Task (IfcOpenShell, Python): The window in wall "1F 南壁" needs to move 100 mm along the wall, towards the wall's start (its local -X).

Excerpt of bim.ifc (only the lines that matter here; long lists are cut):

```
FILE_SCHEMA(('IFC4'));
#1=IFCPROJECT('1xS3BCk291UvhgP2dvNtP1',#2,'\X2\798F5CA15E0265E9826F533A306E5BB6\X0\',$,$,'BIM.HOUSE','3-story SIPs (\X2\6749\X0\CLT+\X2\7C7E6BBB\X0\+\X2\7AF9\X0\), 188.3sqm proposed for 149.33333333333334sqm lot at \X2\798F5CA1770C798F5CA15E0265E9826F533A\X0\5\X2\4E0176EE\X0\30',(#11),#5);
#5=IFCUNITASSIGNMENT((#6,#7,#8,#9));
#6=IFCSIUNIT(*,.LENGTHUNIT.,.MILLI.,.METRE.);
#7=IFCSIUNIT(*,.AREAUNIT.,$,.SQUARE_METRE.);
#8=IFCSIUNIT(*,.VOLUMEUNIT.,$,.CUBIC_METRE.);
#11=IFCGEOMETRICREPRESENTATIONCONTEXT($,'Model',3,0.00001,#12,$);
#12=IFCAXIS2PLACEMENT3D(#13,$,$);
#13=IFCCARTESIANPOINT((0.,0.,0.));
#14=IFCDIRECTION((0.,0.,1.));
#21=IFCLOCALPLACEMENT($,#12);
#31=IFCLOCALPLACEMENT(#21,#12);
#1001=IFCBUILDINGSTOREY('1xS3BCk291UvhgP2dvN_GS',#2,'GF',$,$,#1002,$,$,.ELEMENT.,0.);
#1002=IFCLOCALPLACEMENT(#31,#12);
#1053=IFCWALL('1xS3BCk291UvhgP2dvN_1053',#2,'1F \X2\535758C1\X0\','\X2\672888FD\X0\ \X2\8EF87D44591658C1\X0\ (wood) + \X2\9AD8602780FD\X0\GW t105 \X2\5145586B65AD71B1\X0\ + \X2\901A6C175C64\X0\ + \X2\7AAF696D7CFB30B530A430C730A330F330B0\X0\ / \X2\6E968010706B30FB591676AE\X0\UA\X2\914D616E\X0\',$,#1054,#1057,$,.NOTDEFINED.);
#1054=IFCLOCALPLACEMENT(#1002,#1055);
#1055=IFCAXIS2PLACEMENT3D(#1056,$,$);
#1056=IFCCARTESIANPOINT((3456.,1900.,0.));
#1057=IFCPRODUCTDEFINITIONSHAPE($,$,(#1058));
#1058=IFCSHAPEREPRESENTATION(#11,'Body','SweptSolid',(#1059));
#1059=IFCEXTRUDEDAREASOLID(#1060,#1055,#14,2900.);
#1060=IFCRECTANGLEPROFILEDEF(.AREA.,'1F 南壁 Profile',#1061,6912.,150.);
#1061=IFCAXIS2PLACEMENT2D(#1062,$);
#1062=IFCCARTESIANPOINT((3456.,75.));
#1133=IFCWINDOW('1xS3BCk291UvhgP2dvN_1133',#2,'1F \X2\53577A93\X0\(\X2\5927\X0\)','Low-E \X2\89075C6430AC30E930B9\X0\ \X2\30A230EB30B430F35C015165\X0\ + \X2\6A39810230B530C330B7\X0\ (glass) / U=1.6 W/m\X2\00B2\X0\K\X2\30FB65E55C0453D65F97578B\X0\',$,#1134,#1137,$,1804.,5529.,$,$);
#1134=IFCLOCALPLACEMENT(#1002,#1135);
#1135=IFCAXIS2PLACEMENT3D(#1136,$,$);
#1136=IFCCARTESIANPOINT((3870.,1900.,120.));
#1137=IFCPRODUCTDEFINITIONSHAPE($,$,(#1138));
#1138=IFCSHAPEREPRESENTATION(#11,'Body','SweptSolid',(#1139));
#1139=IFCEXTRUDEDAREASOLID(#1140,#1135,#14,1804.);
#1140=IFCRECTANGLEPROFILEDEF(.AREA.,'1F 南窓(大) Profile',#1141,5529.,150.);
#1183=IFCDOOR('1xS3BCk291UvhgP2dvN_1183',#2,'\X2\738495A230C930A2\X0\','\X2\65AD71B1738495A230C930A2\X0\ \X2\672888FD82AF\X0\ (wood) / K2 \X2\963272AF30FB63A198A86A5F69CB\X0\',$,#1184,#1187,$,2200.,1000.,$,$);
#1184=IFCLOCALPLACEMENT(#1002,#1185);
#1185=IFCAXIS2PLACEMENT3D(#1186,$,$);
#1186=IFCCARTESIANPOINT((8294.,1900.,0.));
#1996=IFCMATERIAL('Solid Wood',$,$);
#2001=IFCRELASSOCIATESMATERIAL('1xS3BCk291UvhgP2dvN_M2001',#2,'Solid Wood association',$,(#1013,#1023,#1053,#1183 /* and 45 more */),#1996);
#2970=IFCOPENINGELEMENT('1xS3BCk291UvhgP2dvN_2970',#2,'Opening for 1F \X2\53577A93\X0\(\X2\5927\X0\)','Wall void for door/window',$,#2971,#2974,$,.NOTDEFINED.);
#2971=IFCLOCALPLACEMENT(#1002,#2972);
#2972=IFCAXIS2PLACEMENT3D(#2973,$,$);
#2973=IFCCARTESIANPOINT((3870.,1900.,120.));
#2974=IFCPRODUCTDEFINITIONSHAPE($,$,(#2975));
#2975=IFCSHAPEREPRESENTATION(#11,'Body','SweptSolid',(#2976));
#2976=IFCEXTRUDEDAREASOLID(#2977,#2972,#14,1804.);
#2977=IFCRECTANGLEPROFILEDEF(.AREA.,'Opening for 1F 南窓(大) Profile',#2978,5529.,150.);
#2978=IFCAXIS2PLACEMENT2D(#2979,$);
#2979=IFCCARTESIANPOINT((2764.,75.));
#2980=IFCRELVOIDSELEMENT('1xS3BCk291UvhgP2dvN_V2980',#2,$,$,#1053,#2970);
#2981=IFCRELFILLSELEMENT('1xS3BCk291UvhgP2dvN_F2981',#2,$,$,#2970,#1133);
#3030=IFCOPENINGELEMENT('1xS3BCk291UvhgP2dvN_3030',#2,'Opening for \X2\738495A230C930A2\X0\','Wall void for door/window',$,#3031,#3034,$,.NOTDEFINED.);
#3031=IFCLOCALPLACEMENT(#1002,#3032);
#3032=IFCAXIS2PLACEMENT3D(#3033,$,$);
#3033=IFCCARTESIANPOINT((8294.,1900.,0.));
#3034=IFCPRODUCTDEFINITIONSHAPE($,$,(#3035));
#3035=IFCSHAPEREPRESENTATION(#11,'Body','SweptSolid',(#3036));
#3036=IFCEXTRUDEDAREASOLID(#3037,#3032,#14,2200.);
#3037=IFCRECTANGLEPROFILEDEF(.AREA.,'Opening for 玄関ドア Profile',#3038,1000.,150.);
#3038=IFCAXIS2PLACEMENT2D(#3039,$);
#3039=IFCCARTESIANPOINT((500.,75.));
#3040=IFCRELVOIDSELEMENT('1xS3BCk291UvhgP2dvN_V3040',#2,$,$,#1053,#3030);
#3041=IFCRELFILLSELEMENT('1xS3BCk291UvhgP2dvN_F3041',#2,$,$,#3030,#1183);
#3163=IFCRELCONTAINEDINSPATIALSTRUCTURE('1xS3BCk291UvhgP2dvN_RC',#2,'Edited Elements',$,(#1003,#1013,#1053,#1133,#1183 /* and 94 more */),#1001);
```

```python
import ifcopenshell
import ifcopenshell.api.geometry
import ifcopenshell.util.placement
import ifcopenshell.util.unit

model = ifcopenshell.open("bim.ifc")
unit_scale = ifcopenshell.util.unit.calculate_unit_scale(model)

window = model.by_id(1133)
opening = window.FillsVoids[0].RelatingOpeningElement
wall = opening.VoidsElements[0].RelatingBuildingElement

wall_matrix = ifcopenshell.util.placement.get_local_placement(wall.ObjectPlacement)
shift = wall_matrix[:3, 0] * -0.1 / unit_scale
before = ifcopenshell.util.placement.get_local_placement(window.ObjectPlacement)[:3, 3].copy()

# The window is not placed relative to its opening, so move both.
for product in (opening, window):
    matrix = ifcopenshell.util.placement.get_local_placement(product.ObjectPlacement)
    matrix[:3, 3] += shift
    ifcopenshell.api.geometry.edit_object_placement(model, product=product, matrix=matrix, is_si=False)

after = ifcopenshell.util.placement.get_local_placement(window.ObjectPlacement)[:3, 3]
print("window moved by", (after - before).round(3) + 0.0)

model.write("bim-out.ifc")
```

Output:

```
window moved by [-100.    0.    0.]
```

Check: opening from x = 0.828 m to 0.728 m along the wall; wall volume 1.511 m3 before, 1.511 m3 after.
